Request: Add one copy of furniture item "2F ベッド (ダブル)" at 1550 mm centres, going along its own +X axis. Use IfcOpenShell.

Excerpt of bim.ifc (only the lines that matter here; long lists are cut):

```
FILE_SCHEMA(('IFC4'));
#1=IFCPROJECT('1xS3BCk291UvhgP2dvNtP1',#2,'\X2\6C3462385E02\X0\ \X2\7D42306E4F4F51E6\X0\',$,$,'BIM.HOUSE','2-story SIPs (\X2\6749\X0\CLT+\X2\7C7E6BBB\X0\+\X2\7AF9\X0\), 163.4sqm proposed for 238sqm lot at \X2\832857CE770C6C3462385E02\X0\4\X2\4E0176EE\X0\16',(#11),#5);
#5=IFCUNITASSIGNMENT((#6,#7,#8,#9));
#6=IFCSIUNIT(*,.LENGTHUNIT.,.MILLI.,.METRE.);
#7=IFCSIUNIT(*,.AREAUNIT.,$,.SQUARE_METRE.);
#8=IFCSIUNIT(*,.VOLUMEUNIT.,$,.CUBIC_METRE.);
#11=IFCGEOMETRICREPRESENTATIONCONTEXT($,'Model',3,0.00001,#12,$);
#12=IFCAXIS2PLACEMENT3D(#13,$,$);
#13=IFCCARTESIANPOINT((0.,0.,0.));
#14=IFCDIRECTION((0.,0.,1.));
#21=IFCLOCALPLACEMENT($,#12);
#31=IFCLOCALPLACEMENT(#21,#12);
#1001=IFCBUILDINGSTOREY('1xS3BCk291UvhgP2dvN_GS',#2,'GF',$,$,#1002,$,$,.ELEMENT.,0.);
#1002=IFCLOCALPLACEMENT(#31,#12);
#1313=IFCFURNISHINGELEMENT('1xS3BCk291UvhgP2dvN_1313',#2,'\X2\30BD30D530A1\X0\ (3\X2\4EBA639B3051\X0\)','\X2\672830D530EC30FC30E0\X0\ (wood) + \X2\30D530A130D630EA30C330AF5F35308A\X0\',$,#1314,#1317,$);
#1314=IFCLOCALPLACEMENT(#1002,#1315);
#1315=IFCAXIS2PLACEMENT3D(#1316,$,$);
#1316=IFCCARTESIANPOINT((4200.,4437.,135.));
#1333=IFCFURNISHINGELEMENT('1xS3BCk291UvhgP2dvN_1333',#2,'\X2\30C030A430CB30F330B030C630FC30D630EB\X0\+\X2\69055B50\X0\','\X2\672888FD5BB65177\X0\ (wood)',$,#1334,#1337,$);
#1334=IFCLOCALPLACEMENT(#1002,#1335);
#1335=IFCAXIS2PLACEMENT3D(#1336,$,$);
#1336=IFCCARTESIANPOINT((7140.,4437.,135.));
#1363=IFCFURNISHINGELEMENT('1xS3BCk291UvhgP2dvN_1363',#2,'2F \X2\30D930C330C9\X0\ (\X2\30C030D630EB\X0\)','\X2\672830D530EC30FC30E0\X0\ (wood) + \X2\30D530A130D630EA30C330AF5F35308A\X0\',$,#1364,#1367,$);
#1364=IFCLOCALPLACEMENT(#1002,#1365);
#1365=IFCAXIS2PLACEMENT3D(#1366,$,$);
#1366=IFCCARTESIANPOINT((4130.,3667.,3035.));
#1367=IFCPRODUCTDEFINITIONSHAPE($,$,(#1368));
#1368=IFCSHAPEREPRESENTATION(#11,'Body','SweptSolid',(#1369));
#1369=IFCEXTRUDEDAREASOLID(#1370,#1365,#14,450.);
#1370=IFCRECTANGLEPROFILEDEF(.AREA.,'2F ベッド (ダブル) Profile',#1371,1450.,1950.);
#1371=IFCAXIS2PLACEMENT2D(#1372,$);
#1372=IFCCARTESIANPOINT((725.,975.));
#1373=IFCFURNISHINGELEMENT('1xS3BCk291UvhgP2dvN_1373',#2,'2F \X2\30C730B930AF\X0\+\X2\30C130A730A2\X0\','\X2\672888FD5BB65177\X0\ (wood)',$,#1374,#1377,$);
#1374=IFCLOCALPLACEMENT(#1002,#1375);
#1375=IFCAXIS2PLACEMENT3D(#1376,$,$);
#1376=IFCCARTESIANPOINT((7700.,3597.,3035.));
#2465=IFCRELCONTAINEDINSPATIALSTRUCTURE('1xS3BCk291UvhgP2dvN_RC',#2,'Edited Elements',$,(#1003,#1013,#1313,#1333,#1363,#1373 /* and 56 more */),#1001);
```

```python
import ifcopenshell
import ifcopenshell.api.geometry
import ifcopenshell.api.root
import ifcopenshell.util.element
import ifcopenshell.util.placement
import ifcopenshell.util.unit

model = ifcopenshell.open("bim.ifc")
unit_scale = ifcopenshell.util.unit.calculate_unit_scale(model)


def reuse_history(source, copy):
    """copy_class also copies each property set's owner history, people and application; keep the originals."""
    for rel in copy.IsDefinedBy:
        if rel.is_a("IfcRelDefinesByProperties") and (history := rel.RelatingPropertyDefinition.OwnerHistory):
            rel.RelatingPropertyDefinition.OwnerHistory = source.OwnerHistory
            ifcopenshell.util.element.remove_deep2(model, history)


source = model.by_id(1363)
base = ifcopenshell.util.placement.get_local_placement(source.ObjectPlacement)
step = base[:3, 0] * 1.55 / unit_scale

for i in range(1, 2):
    copy = ifcopenshell.api.root.copy_class(model, product=source)
    copy.Representation = ifcopenshell.util.element.copy_deep(
        model, source.Representation, exclude=["IfcGeometricRepresentationContext", "IfcRepresentationMap"]
    )
    reuse_history(source, copy)
    matrix = base.copy()
    matrix[:3, 3] += i * step
    print("added at", matrix[:3, 3].round(3) + 0.0)
    ifcopenshell.api.geometry.edit_object_placement(model, product=copy, matrix=matrix, is_si=False)

model.write("bim_updated.ifc")
```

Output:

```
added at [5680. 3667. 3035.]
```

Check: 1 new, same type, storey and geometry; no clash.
